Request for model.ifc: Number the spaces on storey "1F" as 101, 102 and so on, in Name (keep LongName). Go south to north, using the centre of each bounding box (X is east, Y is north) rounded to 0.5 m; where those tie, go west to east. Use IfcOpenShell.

First a look at what the model holds.

```python
import ifcopenshell
import ifcopenshell.util.element
import ifcopenshell.util.placement

model = ifcopenshell.open("model.ifc")
print(model.schema)
storey = next(s for s in model.by_type("IfcBuildingStorey") if s.Name == "1F")
spaces = [e for e in ifcopenshell.util.element.get_decomposition(storey) if e.is_a("IfcSpace")]
for e in sorted(spaces, key=lambda e: e.id()):
    origin = ifcopenshell.util.placement.get_local_placement(e.ObjectPlacement)[:3, 3]
    print(e.id(), e.Name, e.LongName, origin.round(2) + 0.0, sep=" | ")
```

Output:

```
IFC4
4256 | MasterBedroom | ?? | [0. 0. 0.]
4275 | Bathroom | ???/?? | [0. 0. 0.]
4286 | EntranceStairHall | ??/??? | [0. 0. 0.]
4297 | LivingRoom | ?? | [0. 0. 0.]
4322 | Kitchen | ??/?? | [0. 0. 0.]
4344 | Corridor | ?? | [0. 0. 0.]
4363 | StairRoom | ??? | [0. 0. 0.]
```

```python
import ifcopenshell
import ifcopenshell.geom
import ifcopenshell.util.element
import ifcopenshell.util.shape

model = ifcopenshell.open("model.ifc")
settings = ifcopenshell.geom.settings()
settings.set("use-world-coords", True)


def centre(element):
    shape = ifcopenshell.geom.create_shape(settings, element)
    return ifcopenshell.util.shape.get_bbox_centroid(shape.geometry)


storey = next(s for s in model.by_type("IfcBuildingStorey") if s.Name == "1F")
spaces = [e for e in ifcopenshell.util.element.get_decomposition(storey) if e.is_a("IfcSpace")]

# Insertion points can sit at a corner or the storey origin, so sort by the geometry (in metres).
centres = {e: centre(e) for e in spaces}
spaces.sort(key=lambda e: (round(centres[e][1] / 0.5), centres[e][0]))

for i, e in enumerate(spaces, start=1):
    number = f"1{i:02d}"
    e.Name = number
    print(e.id(), number)

model.write("model_edited.ifc")
```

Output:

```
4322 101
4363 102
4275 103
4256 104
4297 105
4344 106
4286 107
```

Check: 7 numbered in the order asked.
